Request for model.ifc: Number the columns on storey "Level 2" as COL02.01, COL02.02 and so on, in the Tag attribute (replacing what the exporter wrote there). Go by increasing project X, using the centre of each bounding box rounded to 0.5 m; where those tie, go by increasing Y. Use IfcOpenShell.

First a look at what the model holds.

```python
import ifcopenshell
import ifcopenshell.util.element
import ifcopenshell.util.placement

model = ifcopenshell.open("model.ifc")
print(model.schema)
storey = next(s for s in model.by_type("IfcBuildingStorey") if s.Name == "Level 2")
columns = [e for e in ifcopenshell.util.element.get_decomposition(storey) if e.is_a("IfcColumn")]
for e in sorted(columns, key=lambda e: e.id()):
    origin = ifcopenshell.util.placement.get_local_placement(e.ObjectPlacement)[:3, 3]
    print(e.id(), e.Tag, e.Name, origin.round(2) + 0.0, sep=" | ")
```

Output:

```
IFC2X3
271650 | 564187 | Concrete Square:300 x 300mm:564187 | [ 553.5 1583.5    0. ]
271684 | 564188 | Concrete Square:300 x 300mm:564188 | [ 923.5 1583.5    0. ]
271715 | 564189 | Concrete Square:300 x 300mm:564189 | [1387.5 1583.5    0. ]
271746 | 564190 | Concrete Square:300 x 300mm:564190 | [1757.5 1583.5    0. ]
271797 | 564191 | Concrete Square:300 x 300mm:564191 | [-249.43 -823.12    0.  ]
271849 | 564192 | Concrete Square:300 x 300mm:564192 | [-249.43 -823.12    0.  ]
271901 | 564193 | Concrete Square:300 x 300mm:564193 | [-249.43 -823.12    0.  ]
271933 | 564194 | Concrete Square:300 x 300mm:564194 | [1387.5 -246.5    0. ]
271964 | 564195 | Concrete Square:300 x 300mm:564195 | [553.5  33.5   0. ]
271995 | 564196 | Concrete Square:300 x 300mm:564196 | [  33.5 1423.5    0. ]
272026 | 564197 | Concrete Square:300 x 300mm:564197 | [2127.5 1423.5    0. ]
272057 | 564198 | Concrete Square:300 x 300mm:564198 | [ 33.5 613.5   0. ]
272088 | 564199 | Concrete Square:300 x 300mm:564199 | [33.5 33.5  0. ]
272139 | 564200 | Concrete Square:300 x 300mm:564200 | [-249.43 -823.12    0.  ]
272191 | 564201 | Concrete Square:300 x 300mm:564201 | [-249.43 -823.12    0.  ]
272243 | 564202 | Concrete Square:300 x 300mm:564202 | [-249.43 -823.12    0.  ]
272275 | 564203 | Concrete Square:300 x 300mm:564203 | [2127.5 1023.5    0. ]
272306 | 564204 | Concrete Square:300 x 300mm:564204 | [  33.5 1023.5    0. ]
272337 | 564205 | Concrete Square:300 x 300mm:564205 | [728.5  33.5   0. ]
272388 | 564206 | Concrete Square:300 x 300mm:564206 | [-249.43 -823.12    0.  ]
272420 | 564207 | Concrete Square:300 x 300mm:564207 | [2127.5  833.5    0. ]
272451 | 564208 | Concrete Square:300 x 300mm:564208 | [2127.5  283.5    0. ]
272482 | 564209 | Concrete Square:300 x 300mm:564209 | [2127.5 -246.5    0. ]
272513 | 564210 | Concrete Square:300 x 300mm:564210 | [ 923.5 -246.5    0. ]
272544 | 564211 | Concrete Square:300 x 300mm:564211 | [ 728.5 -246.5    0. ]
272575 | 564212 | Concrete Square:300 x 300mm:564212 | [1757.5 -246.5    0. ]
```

```python
import ifcopenshell
import ifcopenshell.geom
import ifcopenshell.util.element
import ifcopenshell.util.shape

model = ifcopenshell.open("model.ifc")
settings = ifcopenshell.geom.settings()
settings.set("use-world-coords", True)


def centre(element):
    shape = ifcopenshell.geom.create_shape(settings, element)
    return ifcopenshell.util.shape.get_bbox_centroid(shape.geometry)


storey = next(s for s in model.by_type("IfcBuildingStorey") if s.Name == "Level 2")
columns = [e for e in ifcopenshell.util.element.get_decomposition(storey) if e.is_a("IfcColumn")]

# Insertion points can sit at a corner or the storey origin, so sort by the geometry (in metres).
centres = {e: centre(e) for e in columns}
columns.sort(key=lambda e: (round(centres[e][0] / 0.5), centres[e][1]))

for i, e in enumerate(columns, start=1):
    number = f"COL02.{i:02d}"
    e.Tag = number
    print(e.id(), number)

model.write("model-out.ifc")
```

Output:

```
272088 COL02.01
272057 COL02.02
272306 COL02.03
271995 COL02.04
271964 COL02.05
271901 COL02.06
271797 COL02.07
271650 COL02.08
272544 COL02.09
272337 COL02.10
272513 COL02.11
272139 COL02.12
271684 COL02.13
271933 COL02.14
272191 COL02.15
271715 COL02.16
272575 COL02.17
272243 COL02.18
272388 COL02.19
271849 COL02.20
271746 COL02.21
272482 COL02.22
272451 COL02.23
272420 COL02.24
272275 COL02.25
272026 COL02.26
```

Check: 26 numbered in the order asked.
